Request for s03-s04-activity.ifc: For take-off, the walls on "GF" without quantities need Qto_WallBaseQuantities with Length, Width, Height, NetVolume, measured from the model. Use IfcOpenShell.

First a look at what the model holds.

```python
import ifcopenshell
import ifcopenshell.util.element
import ifcopenshell.util.unit

model = ifcopenshell.open("s03-s04-activity.ifc")
print(model.schema)
for unit_type in ("LENGTHUNIT", "AREAUNIT", "VOLUMEUNIT"):
    print(unit_type, ifcopenshell.util.unit.calculate_unit_scale(model, unit_type))
storey = next(s for s in model.by_type("IfcBuildingStorey") if s.Name == "GF")
walls = [e for e in ifcopenshell.util.element.get_decomposition(storey) if e.is_a("IfcWall")]
for e in sorted(walls, key=lambda e: e.id()):
    print(e.id(), e.is_a(), e.Name, list(ifcopenshell.util.element.get_psets(e, qtos_only=True)), sep=" | ")
```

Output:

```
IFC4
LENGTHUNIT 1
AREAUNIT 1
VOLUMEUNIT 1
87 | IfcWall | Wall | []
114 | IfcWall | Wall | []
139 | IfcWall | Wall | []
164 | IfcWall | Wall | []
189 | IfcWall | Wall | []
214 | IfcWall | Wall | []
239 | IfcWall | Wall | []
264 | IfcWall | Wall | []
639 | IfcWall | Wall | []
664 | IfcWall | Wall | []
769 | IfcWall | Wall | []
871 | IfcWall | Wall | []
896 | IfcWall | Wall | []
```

```python
import ifcopenshell
import ifcopenshell.api.pset
import ifcopenshell.geom
import ifcopenshell.util.element
import ifcopenshell.util.shape
import ifcopenshell.util.unit

model = ifcopenshell.open("s03-s04-activity.ifc")
unit_scale = ifcopenshell.util.unit.calculate_unit_scale(model)
volume_scale = ifcopenshell.util.unit.calculate_unit_scale(model, "VOLUMEUNIT")
settings = ifcopenshell.geom.settings()

storey = next(s for s in model.by_type("IfcBuildingStorey") if s.Name == "GF")
walls = [e for e in ifcopenshell.util.element.get_decomposition(storey) if e.is_a("IfcWall")]

for e in sorted(walls, key=lambda e: e.id()):
    if ifcopenshell.util.element.get_psets(e, qtos_only=True, should_inherit=False):
        continue
    # Geometry comes back in metres, in the element's own axes.
    shape = ifcopenshell.geom.create_shape(settings, e)
    values = {
        "Length": ifcopenshell.util.shape.get_x(shape.geometry) / unit_scale,
        "Width": ifcopenshell.util.shape.get_y(shape.geometry) / unit_scale,
        "Height": ifcopenshell.util.shape.get_z(shape.geometry) / unit_scale,
        "NetVolume": ifcopenshell.util.shape.get_volume(shape.geometry) / volume_scale,
    }
    qto = ifcopenshell.api.pset.add_qto(model, product=e, name="Qto_WallBaseQuantities")
    ifcopenshell.api.pset.edit_qto(model, qto=qto, properties=values)
    print(e.id(), {k: round(v, 3) for k, v in values.items()})

model.write("s03-s04-activity_v2.ifc")
```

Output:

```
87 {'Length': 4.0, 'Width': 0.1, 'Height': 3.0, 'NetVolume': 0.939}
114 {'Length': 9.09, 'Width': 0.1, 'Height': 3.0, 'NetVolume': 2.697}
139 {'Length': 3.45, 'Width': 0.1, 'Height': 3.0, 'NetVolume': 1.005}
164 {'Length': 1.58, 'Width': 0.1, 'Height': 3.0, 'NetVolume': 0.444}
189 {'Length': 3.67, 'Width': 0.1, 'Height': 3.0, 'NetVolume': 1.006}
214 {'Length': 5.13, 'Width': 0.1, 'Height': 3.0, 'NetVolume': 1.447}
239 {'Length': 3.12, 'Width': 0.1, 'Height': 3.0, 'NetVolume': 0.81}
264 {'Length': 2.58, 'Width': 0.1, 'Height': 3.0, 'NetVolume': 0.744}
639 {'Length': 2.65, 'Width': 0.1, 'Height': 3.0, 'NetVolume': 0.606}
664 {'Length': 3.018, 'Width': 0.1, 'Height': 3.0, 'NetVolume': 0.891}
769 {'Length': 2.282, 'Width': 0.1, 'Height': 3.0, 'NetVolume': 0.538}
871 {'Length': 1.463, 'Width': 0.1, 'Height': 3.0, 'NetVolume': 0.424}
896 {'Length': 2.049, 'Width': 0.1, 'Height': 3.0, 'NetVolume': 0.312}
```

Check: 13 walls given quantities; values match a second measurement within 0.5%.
